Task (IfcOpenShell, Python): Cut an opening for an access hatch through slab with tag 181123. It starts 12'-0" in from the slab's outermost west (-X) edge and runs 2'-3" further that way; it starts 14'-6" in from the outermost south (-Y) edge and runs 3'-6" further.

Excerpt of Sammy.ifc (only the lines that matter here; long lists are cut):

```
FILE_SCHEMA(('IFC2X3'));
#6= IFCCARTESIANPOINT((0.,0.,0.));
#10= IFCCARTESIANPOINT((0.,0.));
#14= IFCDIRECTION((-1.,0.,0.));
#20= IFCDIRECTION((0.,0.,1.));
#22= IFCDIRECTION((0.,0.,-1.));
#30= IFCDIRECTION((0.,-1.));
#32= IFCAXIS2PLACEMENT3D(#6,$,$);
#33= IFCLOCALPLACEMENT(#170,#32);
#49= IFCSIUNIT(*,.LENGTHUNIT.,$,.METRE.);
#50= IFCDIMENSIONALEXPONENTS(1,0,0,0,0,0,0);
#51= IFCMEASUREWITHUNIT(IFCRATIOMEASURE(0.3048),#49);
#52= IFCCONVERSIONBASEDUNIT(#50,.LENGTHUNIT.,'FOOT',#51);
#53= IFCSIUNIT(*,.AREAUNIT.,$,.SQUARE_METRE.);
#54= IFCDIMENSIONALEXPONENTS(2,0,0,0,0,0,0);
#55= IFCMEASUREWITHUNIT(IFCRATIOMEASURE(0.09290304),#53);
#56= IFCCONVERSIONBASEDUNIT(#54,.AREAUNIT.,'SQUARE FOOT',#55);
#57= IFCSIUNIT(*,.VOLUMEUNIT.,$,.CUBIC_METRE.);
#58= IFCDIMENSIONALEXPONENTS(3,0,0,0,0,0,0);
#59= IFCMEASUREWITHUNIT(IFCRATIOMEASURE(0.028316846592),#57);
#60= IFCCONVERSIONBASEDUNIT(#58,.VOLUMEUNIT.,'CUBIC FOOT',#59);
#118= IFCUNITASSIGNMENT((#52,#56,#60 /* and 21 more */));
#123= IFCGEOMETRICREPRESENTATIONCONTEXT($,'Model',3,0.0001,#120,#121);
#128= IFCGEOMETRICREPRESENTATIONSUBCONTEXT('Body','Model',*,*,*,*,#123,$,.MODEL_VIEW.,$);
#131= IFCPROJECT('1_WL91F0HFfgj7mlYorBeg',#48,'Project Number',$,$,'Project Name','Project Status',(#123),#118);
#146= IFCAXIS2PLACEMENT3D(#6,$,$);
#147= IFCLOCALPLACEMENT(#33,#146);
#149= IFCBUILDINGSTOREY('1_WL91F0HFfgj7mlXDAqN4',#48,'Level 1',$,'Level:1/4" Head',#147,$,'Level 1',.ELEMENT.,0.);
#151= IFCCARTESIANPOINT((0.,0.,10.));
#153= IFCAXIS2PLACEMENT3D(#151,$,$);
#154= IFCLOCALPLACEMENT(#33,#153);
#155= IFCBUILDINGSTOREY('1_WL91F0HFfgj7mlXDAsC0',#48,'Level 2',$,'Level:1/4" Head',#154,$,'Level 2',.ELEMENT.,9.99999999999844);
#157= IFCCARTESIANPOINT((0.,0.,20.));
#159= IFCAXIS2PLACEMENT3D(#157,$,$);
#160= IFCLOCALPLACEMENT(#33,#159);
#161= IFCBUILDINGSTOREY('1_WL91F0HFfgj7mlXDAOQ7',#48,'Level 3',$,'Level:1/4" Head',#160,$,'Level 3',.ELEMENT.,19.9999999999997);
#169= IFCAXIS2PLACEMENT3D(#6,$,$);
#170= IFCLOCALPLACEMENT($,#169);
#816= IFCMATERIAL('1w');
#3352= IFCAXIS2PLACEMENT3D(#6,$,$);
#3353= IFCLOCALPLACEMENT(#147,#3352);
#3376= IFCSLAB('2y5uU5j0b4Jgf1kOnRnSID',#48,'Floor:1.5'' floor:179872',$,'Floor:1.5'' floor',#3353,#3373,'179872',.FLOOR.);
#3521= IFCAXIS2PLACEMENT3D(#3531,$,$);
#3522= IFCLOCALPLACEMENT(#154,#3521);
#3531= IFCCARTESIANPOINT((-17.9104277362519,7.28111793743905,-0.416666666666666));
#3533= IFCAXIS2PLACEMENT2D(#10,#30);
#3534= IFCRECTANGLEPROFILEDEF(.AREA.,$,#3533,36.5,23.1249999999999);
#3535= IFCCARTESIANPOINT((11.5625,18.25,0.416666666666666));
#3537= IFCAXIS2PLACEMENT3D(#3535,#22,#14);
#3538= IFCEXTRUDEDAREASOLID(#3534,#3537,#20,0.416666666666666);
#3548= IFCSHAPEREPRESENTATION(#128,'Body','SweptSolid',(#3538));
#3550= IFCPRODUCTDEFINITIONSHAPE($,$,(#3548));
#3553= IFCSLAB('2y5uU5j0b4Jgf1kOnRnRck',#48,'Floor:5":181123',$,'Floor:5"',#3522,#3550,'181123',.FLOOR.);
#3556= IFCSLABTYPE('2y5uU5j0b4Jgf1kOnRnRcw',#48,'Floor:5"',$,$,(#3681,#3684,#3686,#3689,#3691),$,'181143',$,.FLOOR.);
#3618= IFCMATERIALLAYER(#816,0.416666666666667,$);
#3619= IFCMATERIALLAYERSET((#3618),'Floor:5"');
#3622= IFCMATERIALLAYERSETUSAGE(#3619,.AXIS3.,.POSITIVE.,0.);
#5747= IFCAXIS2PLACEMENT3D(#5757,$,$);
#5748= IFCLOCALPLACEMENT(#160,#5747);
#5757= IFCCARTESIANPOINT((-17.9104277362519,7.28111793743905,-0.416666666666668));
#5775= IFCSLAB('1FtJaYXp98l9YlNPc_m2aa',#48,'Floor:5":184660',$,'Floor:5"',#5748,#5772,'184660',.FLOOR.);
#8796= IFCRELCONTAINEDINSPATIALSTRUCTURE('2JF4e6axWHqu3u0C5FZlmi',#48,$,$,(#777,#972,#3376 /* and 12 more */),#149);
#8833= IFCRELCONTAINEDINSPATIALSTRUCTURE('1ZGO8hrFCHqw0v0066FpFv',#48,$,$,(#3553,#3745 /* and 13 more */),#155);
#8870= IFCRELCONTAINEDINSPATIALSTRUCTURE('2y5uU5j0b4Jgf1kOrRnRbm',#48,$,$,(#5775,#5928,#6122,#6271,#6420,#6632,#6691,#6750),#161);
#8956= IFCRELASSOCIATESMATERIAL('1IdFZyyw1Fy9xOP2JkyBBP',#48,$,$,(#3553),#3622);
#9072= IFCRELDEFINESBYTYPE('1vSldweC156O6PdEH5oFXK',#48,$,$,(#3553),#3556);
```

```python
import numpy as np
import ifcopenshell
import ifcopenshell.api.feature
import ifcopenshell.api.geometry
import ifcopenshell.api.root
import ifcopenshell.geom
import ifcopenshell.util.placement
import ifcopenshell.util.representation
import ifcopenshell.util.shape
import ifcopenshell.util.unit

model = ifcopenshell.open("Sammy.ifc")
unit_scale = ifcopenshell.util.unit.calculate_unit_scale(model)
settings = ifcopenshell.geom.settings()


def volume(element):
    """Net volume in cubic metres, openings subtracted."""
    shape = ifcopenshell.geom.create_shape(settings, element)
    return ifcopenshell.util.shape.get_volume(shape.geometry)


slab = model.by_guid("2y5uU5j0b4Jgf1kOnRnRck")
before = volume(slab)

# Extent in the slab's own axes, in metres. The edges named are its -X and -Y sides.
slab_shape = ifcopenshell.geom.create_shape(settings, slab)
vertices = ifcopenshell.util.shape.get_vertices(slab_shape.geometry)
x_min, y_min, bottom = vertices.min(axis=0)
top = vertices[:, 2].max()

opening = ifcopenshell.api.root.create_entity(model, ifc_class="IfcOpeningElement", name="Access hatch opening")
context = ifcopenshell.util.representation.get_context(model, "Model", "Body", "MODEL_VIEW")
width, depth = 0.6858, 1.0668
outline = [(0.0, 0.0), (width, 0.0), (width, depth), (0.0, depth), (0.0, 0.0)]
# Overshoot both faces by 50 mm so the cut is clean.
shape = ifcopenshell.api.geometry.add_slab_representation(
    model, context=context, depth=top - bottom + 0.1, polyline=outline
)
ifcopenshell.api.geometry.assign_representation(model, product=opening, representation=shape)

matrix = ifcopenshell.util.placement.get_local_placement(slab.ObjectPlacement)
matrix[:, 3] = matrix @ np.append(np.array([x_min + 3.6576, y_min + 4.4196, bottom - 0.05]) / unit_scale, 1.0)
ifcopenshell.api.geometry.edit_object_placement(model, product=opening, matrix=matrix, is_si=False)
ifcopenshell.api.feature.add_feature(model, feature=opening, element=slab)

after = volume(slab)

print(f"slab volume {before:.3f} -> {after:.3f} m3")

model.write("Sammy_edited.ifc")
```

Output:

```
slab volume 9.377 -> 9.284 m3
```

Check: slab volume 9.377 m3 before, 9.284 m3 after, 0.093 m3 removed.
